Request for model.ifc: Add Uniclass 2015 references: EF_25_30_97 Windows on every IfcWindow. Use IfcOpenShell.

First a look at what the model holds.

```python
import ifcopenshell

model = ifcopenshell.open("model.ifc")
print(model.schema)
print("classifications:", [c.Name for c in model.by_type("IfcClassification")])
for ifc_class in ("IfcDoor", "IfcRoof", "IfcStair", "IfcWall", "IfcWindow"):
    print(ifc_class, len(model.by_type(ifc_class)))
```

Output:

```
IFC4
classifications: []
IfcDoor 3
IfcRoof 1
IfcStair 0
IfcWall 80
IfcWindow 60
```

```python
import ifcopenshell
import ifcopenshell.api.classification

model = ifcopenshell.open("model.ifc")

system = ifcopenshell.api.classification.add_classification(model, classification="Uniclass 2015")

codes = {
    "IfcWindow": ("EF_25_30_97", "Windows"),
}
for ifc_class, (code, name) in codes.items():
    products = model.by_type(ifc_class)
    ifcopenshell.api.classification.add_reference(
        model, products=products, classification=system, identification=code, name=name
    )
    print(code, len(products))

model.write("model_rev.ifc")
```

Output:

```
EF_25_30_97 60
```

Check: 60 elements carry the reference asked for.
